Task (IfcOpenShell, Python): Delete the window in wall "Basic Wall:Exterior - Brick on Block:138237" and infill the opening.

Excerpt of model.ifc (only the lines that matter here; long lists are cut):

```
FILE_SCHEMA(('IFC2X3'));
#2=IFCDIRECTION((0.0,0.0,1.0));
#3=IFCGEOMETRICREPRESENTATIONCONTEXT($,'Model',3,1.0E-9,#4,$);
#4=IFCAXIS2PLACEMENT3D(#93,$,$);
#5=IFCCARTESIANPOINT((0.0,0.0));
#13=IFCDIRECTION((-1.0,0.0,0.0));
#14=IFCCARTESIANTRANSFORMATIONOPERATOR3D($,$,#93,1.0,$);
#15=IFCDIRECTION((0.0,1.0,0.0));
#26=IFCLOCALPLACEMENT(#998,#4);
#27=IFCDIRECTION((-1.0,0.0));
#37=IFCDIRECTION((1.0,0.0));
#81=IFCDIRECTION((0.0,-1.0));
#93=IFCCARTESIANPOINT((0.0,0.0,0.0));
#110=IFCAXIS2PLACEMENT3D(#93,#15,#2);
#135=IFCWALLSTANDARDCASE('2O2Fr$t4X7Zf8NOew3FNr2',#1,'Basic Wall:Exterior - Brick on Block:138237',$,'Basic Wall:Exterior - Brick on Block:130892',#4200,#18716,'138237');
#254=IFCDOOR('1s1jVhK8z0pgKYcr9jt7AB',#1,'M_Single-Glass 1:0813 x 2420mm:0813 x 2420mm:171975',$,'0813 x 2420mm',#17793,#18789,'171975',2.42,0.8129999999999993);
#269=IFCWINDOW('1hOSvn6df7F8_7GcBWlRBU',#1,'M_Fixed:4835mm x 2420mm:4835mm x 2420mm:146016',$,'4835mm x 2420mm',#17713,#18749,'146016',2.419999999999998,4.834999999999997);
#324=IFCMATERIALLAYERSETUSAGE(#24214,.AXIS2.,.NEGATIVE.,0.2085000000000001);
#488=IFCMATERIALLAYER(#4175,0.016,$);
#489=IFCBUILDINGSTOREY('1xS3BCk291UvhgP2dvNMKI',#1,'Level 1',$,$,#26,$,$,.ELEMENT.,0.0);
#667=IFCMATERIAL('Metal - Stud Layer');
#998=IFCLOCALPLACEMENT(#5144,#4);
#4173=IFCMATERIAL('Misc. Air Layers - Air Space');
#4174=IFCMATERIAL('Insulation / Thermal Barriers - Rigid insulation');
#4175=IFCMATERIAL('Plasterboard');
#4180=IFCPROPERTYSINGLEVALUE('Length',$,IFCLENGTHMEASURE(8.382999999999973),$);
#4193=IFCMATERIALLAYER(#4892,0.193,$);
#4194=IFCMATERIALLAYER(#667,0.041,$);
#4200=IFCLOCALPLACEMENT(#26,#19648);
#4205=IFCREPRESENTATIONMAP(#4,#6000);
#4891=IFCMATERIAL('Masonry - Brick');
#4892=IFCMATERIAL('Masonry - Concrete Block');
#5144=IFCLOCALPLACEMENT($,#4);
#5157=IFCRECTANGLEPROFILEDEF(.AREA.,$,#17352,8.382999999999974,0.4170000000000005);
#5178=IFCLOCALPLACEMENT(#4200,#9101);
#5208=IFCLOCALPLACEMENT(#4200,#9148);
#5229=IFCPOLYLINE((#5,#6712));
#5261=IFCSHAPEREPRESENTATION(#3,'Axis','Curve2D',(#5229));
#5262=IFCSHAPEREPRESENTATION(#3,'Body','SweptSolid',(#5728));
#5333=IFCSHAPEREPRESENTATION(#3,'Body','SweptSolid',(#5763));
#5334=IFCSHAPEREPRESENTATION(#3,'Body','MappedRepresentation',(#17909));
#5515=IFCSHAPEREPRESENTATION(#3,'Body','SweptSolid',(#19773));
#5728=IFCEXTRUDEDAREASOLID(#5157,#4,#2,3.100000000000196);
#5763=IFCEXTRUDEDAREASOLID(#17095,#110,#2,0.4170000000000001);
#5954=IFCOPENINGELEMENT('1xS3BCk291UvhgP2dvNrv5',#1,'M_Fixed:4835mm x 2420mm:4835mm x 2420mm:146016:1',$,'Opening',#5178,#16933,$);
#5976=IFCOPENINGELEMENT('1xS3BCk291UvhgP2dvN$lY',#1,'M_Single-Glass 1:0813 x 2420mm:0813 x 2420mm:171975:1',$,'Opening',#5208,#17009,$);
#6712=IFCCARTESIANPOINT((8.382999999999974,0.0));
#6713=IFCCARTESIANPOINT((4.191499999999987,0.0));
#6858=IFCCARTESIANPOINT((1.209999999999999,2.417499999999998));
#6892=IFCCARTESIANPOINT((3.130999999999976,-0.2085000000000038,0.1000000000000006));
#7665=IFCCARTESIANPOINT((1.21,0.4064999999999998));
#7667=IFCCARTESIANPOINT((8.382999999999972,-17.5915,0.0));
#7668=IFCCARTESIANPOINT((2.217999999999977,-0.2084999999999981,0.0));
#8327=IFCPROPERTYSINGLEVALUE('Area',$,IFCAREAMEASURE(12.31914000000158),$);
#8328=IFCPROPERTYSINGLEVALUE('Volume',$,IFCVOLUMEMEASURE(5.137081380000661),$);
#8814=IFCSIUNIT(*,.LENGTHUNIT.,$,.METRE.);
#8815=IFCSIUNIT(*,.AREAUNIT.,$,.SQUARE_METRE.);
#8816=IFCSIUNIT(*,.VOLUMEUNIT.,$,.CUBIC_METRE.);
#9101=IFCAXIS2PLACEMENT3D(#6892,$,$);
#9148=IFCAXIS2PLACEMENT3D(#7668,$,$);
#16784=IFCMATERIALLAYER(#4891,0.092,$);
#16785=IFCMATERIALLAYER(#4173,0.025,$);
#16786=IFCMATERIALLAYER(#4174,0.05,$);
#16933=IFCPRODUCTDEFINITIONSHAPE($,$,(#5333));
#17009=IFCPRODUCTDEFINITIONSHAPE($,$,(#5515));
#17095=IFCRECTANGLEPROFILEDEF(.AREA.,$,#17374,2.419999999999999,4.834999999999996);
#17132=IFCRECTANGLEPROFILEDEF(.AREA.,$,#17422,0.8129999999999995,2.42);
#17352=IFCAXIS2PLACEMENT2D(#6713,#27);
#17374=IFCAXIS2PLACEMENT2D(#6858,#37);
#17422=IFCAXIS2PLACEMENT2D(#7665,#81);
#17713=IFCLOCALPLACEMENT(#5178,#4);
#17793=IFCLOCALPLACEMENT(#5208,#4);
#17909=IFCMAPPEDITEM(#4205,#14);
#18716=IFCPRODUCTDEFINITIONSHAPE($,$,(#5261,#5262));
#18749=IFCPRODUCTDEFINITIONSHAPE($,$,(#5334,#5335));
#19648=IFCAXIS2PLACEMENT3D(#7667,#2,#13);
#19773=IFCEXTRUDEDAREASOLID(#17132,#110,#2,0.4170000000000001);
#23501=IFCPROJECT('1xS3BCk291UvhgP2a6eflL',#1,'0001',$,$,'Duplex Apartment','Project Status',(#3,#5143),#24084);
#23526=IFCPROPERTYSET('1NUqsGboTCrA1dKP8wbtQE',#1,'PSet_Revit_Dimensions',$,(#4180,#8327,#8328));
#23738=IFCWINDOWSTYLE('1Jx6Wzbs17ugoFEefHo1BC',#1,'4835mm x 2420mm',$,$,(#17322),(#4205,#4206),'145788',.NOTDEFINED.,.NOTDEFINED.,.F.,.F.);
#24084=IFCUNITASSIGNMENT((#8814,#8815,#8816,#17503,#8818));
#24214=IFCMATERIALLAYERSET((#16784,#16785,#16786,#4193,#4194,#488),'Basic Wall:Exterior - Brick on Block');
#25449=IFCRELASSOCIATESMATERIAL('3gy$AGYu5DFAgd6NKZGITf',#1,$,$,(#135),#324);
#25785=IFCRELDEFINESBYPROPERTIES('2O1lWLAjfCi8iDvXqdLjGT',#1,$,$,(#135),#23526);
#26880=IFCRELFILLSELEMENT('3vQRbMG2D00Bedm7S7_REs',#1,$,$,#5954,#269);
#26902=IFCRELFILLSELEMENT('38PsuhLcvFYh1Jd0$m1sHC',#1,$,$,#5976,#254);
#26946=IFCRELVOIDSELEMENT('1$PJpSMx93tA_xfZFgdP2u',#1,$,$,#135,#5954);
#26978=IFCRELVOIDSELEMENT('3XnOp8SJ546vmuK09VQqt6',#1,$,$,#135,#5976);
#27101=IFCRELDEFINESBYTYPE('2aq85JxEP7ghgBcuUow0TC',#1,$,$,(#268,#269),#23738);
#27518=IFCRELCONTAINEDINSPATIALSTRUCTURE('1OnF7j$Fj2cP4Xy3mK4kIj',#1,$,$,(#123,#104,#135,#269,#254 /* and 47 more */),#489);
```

```python
import ifcopenshell
import ifcopenshell.api.feature
import ifcopenshell.api.pset
import ifcopenshell.api.root
import ifcopenshell.geom
import ifcopenshell.util.element
import ifcopenshell.util.shape
import ifcopenshell.util.unit

model = ifcopenshell.open("model.ifc")
area_scale = ifcopenshell.util.unit.calculate_unit_scale(model, "AREAUNIT")
volume_scale = ifcopenshell.util.unit.calculate_unit_scale(model, "VOLUMEUNIT")
settings = ifcopenshell.geom.settings()


def volume(element):
    """Net volume in cubic metres, openings subtracted."""
    shape = ifcopenshell.geom.create_shape(settings, element)
    return ifcopenshell.util.shape.get_volume(shape.geometry)


window = model.by_guid("1hOSvn6df7F8_7GcBWlRBU")
opening = window.FillsVoids[0].RelatingOpeningElement
wall = opening.VoidsElements[0].RelatingBuildingElement
before = volume(wall)

ifcopenshell.api.root.remove_product(model, product=window)
ifcopenshell.api.feature.remove_feature(model, feature=opening)

after = volume(wall)
thickness = 0.417  # wall thickness in metres

# Update the wall's stored quantities.
pset = model.by_id(ifcopenshell.util.element.get_pset(wall, "PSet_Revit_Dimensions", should_inherit=False)["id"])
ifcopenshell.api.pset.edit_pset(model, pset=pset, properties={
    "Area": model.create_entity("IfcAreaMeasure", after / thickness / area_scale),
    "Volume": model.create_entity("IfcVolumeMeasure", after / volume_scale),
})

print(f"wall volume {before:.3f} -> {after:.3f} m3")

model.write("model_edited.ifc")
```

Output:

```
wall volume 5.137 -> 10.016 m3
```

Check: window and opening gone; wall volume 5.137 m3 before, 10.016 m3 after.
